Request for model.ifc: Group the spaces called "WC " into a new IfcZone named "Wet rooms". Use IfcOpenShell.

First a look at what the model holds.

```python
import ifcopenshell

model = ifcopenshell.open("model.ifc")
print(model.schema)
seen = {}
for space in model.by_type("IfcSpace"):
    seen[space.LongName] = seen.get(space.LongName, 0) + 1
for name, count in sorted(seen.items(), key=str):
    print(count, "x", name)
print("zones:", [z.Name for z in model.by_type("IfcZone")][:20])
```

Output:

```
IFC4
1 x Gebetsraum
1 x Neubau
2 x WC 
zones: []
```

```python
import ifcopenshell
import ifcopenshell.api.group
import ifcopenshell.api.root

model = ifcopenshell.open("model.ifc")

names = {"WC "}
spaces = [s for s in model.by_type("IfcSpace") if s.LongName in names]

zone = ifcopenshell.api.root.create_entity(model, ifc_class="IfcZone", name="Wet rooms")
ifcopenshell.api.group.assign_group(model, products=spaces, group=zone)
print(len(spaces), "spaces in", zone.Name)

model.write("model_v2.ifc")
```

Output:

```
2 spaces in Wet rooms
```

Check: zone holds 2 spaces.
